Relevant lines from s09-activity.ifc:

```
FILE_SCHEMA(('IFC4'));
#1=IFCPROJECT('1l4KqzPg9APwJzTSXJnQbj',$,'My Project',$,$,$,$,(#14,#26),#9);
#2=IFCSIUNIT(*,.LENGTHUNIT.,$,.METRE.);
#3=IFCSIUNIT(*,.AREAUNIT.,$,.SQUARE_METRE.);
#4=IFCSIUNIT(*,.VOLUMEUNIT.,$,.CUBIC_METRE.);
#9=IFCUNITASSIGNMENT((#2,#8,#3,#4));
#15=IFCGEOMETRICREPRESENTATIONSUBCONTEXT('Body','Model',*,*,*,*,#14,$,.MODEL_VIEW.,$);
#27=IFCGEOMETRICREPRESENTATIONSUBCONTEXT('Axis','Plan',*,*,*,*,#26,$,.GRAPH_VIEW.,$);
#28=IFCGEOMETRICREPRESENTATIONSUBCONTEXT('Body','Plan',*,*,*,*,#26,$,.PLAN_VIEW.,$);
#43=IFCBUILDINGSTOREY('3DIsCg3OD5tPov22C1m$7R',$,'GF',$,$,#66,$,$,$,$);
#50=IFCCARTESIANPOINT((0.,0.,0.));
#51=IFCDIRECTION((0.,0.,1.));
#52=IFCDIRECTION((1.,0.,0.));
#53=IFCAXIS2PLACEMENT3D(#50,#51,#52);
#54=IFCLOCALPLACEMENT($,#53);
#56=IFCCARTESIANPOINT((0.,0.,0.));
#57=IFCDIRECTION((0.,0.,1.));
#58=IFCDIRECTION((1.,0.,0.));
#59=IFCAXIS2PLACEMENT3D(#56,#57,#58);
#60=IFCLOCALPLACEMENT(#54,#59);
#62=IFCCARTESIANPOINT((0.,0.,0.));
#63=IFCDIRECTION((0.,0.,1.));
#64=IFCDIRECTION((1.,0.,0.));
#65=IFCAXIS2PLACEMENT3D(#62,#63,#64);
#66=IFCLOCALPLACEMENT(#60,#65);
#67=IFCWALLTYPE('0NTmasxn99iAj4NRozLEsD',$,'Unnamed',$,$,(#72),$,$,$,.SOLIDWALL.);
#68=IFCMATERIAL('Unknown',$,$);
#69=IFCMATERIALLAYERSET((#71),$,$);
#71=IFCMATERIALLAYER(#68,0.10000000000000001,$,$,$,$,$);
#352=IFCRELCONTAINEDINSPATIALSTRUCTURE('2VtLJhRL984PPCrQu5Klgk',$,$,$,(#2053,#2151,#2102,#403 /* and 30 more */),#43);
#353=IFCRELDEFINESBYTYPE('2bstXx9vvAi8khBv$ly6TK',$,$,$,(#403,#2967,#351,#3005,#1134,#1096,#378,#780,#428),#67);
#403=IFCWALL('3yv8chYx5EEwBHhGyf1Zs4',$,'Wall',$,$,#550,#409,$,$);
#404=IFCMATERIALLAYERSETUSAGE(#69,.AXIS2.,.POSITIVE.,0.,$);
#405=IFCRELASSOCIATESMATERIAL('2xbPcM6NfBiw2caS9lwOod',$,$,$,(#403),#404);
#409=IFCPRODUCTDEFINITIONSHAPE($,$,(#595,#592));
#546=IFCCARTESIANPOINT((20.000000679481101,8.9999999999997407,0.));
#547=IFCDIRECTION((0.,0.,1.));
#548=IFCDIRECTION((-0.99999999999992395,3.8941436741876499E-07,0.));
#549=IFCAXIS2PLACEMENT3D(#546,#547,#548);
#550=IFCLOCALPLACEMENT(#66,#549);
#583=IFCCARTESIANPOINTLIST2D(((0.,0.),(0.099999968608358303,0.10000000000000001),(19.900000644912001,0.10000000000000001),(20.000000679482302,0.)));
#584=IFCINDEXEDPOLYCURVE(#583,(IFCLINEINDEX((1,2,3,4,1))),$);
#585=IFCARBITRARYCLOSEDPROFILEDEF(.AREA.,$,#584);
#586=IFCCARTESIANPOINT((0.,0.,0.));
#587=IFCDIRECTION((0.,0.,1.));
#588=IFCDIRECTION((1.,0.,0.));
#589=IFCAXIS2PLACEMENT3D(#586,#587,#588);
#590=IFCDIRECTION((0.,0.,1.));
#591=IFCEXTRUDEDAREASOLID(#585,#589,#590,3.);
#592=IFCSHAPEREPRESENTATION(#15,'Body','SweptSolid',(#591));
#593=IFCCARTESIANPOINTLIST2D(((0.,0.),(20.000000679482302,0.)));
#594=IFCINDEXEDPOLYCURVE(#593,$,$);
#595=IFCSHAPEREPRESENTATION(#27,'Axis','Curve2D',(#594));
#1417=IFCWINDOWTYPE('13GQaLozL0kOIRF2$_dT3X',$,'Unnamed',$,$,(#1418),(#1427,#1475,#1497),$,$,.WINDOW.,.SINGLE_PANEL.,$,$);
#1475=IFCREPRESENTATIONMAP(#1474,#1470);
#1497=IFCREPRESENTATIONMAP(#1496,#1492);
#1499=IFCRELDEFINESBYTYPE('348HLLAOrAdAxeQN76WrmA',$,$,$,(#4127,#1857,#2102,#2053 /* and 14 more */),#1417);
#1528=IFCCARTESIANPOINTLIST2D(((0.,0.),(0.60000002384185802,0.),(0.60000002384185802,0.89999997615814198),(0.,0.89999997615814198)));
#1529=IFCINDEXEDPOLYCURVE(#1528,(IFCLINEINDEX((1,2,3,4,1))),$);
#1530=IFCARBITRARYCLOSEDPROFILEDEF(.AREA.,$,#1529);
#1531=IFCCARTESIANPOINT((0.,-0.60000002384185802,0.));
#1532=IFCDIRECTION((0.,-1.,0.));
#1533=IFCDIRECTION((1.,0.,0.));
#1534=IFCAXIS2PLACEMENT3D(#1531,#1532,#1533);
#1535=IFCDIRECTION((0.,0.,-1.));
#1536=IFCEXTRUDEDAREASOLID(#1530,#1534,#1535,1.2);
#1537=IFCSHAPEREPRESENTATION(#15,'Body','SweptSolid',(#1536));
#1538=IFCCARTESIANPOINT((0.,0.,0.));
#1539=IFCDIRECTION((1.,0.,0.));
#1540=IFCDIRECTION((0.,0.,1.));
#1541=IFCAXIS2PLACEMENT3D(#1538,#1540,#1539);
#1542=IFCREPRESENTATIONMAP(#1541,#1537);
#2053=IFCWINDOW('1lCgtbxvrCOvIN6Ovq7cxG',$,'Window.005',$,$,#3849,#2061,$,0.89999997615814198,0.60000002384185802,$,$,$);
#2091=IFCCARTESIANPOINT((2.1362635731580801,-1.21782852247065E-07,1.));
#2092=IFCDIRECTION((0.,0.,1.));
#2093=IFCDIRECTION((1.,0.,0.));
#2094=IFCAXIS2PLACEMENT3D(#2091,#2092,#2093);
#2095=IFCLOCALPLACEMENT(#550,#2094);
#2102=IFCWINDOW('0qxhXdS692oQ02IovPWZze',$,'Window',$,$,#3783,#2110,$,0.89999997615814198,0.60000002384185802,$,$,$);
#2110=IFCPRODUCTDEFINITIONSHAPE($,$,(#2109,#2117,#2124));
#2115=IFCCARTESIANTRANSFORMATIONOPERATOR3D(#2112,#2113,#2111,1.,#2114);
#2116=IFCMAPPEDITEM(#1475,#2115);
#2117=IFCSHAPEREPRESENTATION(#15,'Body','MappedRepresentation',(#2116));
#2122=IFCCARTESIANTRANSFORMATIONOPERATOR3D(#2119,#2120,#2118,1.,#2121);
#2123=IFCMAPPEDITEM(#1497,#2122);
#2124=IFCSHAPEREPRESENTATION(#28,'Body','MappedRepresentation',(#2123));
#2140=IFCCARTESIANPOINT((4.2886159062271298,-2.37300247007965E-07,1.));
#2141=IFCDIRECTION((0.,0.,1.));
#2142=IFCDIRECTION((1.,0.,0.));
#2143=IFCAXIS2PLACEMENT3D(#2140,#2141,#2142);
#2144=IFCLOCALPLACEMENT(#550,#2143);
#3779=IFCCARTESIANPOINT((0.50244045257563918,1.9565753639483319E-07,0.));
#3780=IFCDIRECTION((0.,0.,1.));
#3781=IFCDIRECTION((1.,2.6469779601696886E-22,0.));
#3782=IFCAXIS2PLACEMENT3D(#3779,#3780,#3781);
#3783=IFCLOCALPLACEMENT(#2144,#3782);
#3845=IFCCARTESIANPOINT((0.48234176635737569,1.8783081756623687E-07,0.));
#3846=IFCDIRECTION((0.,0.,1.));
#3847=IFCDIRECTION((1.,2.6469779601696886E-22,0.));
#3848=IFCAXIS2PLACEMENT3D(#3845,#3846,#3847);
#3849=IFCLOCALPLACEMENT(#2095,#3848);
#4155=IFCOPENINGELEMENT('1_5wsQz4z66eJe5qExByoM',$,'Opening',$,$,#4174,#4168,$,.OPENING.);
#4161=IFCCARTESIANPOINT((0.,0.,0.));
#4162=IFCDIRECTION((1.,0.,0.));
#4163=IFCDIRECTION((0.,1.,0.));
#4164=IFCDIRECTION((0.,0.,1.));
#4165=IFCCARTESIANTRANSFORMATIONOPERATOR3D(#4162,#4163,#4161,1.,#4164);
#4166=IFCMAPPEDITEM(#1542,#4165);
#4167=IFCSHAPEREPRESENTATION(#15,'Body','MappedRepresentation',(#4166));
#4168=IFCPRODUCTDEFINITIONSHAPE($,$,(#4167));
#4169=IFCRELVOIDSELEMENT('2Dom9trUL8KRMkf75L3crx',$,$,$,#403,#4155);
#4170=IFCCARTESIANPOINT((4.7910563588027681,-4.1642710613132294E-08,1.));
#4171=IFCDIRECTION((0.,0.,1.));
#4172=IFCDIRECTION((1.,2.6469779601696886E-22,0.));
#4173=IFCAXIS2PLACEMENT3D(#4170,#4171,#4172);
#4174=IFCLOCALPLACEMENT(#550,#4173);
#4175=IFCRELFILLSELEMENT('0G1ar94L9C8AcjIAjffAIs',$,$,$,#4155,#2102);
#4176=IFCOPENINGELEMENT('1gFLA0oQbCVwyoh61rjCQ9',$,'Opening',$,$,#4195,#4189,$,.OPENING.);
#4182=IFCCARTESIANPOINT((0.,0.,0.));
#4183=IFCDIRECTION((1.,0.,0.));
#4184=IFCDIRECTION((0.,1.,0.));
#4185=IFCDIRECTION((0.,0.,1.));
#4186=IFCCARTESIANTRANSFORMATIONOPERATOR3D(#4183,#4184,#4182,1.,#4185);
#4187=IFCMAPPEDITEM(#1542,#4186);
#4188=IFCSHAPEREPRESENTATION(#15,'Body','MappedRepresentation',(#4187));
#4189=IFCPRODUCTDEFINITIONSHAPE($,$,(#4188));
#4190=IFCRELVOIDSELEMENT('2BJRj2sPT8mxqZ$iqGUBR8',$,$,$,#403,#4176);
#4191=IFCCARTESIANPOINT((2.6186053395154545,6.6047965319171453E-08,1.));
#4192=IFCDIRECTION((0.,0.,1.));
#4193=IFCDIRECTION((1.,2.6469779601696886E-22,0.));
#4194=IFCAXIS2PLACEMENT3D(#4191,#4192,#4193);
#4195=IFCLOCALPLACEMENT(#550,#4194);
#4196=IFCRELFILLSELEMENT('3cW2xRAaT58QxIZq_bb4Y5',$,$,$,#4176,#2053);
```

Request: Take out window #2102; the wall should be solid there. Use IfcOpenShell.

```python
import ifcopenshell
import ifcopenshell.api.feature
import ifcopenshell.api.root
import ifcopenshell.geom
import ifcopenshell.util.shape

model = ifcopenshell.open("s09-activity.ifc")
settings = ifcopenshell.geom.settings()


def volume(element):
    """Net volume in cubic metres, openings subtracted."""
    shape = ifcopenshell.geom.create_shape(settings, element)
    return ifcopenshell.util.shape.get_volume(shape.geometry)


window = model.by_guid("0qxhXdS692oQ02IovPWZze")
opening = window.FillsVoids[0].RelatingOpeningElement
wall = opening.VoidsElements[0].RelatingBuildingElement
before = volume(wall)

ifcopenshell.api.root.remove_product(model, product=window)
ifcopenshell.api.feature.remove_feature(model, feature=opening)

after = volume(wall)

print(f"wall volume {before:.3f} -> {after:.3f} m3")

model.write("s09-activity_v2.ifc")
```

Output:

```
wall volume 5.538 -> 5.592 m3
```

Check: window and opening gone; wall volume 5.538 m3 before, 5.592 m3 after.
